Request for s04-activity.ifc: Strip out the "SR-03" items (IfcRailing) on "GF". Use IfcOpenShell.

First a look at what the model holds.

```python
import ifcopenshell
import ifcopenshell.util.element

model = ifcopenshell.open("s04-activity.ifc")
print(model.schema)
storey = next(s for s in model.by_type("IfcBuildingStorey") if s.Name == "GF")
railings = [e for e in ifcopenshell.util.element.get_decomposition(storey) if e.is_a("IfcRailing")]
seen = {}
for e in railings:
    element_type = ifcopenshell.util.element.get_type(e)
    name = element_type.Name if element_type not in (None, e) else None
    seen[name] = seen.get(name, 0) + 1
for name, count in sorted(seen.items(), key=str):
    print(count, "x", name)
```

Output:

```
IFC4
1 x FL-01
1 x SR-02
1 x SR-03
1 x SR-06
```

```python
import ifcopenshell
import ifcopenshell.api.root
import ifcopenshell.util.element

model = ifcopenshell.open("s04-activity.ifc")

storey = next(s for s in model.by_type("IfcBuildingStorey") if s.Name == "GF")
railings = [e for e in ifcopenshell.util.element.get_decomposition(storey) if e.is_a("IfcRailing")]
targets = [e for e in railings if (t := ifcopenshell.util.element.get_type(e)) not in (None, e) and t.Name == "SR-03"]

for e in targets:
    ifcopenshell.api.root.remove_product(model, product=e)
print(len(targets), "removed")

model.write("s04-activity_v2.ifc")
```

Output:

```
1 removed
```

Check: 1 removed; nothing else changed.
